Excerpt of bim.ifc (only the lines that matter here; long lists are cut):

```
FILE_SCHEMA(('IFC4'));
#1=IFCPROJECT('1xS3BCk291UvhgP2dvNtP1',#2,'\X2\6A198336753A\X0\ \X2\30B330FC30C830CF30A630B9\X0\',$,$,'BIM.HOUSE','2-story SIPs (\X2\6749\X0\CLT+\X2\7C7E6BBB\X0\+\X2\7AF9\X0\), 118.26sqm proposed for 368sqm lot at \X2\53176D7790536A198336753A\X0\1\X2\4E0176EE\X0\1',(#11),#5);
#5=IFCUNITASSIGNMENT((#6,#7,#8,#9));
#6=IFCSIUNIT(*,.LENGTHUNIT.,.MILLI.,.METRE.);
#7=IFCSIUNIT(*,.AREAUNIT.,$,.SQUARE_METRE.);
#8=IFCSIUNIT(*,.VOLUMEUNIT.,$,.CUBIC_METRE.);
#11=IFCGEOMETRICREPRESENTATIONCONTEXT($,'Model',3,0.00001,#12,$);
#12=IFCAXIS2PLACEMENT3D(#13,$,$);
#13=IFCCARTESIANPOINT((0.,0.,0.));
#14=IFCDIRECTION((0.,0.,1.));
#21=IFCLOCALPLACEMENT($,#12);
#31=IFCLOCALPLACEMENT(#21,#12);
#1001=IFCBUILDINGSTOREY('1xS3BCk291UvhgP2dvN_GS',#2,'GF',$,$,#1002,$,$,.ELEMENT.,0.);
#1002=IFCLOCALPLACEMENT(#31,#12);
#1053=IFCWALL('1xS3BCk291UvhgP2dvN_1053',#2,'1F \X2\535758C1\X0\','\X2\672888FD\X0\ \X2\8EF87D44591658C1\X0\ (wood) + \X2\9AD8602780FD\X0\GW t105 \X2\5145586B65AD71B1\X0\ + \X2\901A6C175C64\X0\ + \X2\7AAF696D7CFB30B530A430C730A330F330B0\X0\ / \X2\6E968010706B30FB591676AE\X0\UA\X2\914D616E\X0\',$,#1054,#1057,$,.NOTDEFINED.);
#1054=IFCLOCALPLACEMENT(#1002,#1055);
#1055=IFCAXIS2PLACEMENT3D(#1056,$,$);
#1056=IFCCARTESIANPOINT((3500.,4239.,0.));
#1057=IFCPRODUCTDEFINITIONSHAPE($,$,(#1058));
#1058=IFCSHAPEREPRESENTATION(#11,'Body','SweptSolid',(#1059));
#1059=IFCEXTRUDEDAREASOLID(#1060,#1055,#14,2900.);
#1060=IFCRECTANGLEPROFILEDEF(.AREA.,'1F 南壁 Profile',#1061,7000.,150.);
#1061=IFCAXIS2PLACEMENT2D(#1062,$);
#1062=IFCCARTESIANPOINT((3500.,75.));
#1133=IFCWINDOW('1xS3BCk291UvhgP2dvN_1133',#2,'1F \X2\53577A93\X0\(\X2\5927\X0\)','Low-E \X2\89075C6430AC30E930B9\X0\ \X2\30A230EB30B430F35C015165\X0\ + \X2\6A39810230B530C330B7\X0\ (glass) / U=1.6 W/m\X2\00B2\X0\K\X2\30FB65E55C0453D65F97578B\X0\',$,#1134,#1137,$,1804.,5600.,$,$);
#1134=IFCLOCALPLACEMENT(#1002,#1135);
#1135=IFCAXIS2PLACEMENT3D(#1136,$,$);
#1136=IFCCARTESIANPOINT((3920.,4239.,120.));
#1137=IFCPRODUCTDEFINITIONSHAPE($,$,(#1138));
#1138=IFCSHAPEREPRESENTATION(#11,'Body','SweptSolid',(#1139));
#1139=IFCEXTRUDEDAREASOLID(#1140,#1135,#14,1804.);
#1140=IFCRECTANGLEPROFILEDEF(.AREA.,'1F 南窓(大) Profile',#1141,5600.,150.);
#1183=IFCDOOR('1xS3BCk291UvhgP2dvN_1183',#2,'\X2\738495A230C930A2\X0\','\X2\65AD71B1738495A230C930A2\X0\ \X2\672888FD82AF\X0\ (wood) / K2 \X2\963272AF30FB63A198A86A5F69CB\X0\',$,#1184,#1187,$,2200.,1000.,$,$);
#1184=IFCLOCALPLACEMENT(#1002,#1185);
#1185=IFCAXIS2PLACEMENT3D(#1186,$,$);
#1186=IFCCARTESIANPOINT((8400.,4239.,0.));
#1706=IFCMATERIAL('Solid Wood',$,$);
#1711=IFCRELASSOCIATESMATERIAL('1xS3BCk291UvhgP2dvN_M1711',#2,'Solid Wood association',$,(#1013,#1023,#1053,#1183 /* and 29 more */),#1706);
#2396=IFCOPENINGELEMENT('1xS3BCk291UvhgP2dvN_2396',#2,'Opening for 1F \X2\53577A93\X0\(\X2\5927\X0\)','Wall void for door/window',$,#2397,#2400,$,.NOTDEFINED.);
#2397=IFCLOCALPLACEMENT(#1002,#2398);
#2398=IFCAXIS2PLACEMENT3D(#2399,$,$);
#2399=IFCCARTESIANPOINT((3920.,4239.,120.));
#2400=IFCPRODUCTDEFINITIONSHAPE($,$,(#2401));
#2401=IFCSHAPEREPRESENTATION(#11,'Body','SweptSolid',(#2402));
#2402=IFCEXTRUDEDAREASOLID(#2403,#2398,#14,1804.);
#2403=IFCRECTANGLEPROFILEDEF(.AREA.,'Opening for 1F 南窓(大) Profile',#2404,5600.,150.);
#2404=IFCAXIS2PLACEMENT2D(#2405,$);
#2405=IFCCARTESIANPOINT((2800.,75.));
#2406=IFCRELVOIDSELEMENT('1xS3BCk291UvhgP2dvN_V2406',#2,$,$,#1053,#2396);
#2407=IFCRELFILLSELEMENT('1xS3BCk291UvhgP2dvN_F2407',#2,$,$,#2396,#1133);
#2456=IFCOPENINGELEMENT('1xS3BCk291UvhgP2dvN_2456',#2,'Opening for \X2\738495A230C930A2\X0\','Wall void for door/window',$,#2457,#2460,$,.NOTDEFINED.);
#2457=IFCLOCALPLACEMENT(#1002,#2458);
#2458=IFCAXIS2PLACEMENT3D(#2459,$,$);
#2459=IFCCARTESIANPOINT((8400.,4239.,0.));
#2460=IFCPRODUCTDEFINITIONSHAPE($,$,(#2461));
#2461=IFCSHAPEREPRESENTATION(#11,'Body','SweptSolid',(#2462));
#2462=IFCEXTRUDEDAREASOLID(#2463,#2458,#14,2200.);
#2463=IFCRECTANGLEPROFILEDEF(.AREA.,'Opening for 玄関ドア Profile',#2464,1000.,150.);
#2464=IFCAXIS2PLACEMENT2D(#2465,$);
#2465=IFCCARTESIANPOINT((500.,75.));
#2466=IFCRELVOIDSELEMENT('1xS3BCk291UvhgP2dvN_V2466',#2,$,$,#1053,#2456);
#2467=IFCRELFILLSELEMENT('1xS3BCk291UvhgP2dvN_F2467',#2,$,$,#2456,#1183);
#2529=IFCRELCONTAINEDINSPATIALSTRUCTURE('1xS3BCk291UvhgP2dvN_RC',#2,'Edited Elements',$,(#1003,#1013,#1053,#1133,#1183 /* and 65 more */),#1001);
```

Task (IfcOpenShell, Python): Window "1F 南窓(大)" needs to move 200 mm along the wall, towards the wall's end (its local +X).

```python
import ifcopenshell
import ifcopenshell.api.geometry
import ifcopenshell.util.placement

model = ifcopenshell.open("bim.ifc")

window = model.by_guid("1xS3BCk291UvhgP2dvN_1133")
opening = window.FillsVoids[0].RelatingOpeningElement
wall = opening.VoidsElements[0].RelatingBuildingElement

wall_matrix = ifcopenshell.util.placement.get_local_placement(wall.ObjectPlacement)
shift = wall_matrix[:3, 0] * 200.0
before = ifcopenshell.util.placement.get_local_placement(window.ObjectPlacement)[:3, 3].copy()

# The window is not placed relative to its opening, so move both.
for product in (opening, window):
    matrix = ifcopenshell.util.placement.get_local_placement(product.ObjectPlacement)
    matrix[:3, 3] += shift
    ifcopenshell.api.geometry.edit_object_placement(model, product=product, matrix=matrix, is_si=False)

after = ifcopenshell.util.placement.get_local_placement(window.ObjectPlacement)[:3, 3]
print("window moved by", (after - before).round(3) + 0.0)

model.write("bim_updated.ifc")
```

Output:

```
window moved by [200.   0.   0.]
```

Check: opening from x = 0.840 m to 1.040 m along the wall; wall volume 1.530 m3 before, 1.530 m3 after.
